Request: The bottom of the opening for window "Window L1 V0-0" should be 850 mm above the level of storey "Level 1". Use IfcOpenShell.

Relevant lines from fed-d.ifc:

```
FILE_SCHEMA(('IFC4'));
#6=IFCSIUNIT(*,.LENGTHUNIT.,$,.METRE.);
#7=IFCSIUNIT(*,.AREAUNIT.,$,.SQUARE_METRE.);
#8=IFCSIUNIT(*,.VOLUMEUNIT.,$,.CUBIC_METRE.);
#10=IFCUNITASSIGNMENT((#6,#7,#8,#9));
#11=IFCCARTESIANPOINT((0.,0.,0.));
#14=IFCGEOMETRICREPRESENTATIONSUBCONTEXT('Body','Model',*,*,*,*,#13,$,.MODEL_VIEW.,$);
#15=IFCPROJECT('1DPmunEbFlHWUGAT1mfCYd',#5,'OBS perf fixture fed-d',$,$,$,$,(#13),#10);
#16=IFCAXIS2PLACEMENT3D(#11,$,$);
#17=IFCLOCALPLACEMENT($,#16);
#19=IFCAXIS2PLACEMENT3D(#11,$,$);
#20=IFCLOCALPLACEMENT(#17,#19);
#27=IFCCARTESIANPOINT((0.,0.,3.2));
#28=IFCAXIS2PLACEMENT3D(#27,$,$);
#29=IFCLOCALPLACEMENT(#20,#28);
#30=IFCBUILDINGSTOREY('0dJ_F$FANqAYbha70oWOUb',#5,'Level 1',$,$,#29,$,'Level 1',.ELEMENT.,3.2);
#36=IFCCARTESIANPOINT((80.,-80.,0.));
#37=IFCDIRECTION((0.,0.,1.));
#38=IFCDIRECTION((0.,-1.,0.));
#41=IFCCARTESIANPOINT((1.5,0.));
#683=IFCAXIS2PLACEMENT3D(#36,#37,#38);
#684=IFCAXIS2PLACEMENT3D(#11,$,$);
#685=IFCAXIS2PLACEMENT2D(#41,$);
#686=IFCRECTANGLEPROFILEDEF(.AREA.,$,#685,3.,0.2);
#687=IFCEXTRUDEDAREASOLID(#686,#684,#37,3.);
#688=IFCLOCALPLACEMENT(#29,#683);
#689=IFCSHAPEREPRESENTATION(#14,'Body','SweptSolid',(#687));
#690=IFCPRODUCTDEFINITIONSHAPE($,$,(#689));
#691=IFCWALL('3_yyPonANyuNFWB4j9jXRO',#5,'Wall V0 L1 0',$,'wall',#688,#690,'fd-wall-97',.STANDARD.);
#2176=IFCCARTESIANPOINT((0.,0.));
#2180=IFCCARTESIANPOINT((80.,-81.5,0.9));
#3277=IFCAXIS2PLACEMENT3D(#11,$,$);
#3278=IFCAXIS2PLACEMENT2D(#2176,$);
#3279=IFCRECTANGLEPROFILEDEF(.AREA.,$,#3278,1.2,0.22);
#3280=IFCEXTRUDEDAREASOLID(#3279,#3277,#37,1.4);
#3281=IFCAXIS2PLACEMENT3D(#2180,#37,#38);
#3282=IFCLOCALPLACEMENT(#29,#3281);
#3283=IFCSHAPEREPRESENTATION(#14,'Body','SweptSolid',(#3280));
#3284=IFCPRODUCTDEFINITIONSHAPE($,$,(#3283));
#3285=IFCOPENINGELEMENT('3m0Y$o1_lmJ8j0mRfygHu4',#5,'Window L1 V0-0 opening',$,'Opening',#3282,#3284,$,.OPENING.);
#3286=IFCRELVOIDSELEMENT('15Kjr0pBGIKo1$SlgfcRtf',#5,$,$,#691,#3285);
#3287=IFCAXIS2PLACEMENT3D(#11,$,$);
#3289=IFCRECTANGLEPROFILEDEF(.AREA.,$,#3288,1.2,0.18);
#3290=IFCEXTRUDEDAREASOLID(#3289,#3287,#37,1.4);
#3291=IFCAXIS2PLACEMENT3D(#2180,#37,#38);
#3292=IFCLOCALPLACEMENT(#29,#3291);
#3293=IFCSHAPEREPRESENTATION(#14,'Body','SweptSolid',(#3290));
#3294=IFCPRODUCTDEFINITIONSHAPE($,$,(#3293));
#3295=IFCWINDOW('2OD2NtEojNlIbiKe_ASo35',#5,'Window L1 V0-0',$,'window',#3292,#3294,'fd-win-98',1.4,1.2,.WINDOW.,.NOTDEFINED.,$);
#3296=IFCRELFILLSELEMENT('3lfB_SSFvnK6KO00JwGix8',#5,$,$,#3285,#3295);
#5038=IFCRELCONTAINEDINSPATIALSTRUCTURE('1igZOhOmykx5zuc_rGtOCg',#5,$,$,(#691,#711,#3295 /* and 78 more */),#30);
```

```python
import numpy as np
import ifcopenshell
import ifcopenshell.api.geometry
import ifcopenshell.geom
import ifcopenshell.util.element
import ifcopenshell.util.placement
import ifcopenshell.util.shape
import ifcopenshell.util.unit

model = ifcopenshell.open("fed-d.ifc")
unit_scale = ifcopenshell.util.unit.calculate_unit_scale(model)

window = model.by_guid("2OD2NtEojNlIbiKe_ASo35")
opening = window.FillsVoids[0].RelatingOpeningElement
storey = ifcopenshell.util.element.get_container(window, ifc_class="IfcBuildingStorey")
level = ifcopenshell.util.placement.get_local_placement(storey.ObjectPlacement)[2, 3]

# The opening's origin need not be at the sill, so measure its lowest point.
shape = ifcopenshell.geom.create_shape(ifcopenshell.geom.settings(), opening)
bottom = ifcopenshell.util.shape.get_shape_bottom_elevation(shape, shape.geometry) / unit_scale
dz = level + 0.85 / unit_scale - bottom

shift = np.array([0.0, 0.0, dz])
# The window is not placed relative to its opening, so move both.
for product in (opening, window):
    matrix = ifcopenshell.util.placement.get_local_placement(product.ObjectPlacement)
    matrix[:3, 3] += shift
    ifcopenshell.api.geometry.edit_object_placement(model, product=product, matrix=matrix, is_si=False)

print(f"moved by {dz * unit_scale:+.3f} m")

model.write("fed-d_updated.ifc")
```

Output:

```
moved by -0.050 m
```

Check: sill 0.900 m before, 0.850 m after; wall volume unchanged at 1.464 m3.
